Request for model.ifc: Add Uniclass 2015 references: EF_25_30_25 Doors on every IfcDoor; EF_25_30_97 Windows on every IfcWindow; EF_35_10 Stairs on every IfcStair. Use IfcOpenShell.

First a look at what the model holds.

```python
import ifcopenshell

model = ifcopenshell.open("model.ifc")
print(model.schema)
print("classifications:", [c.Name for c in model.by_type("IfcClassification")])
for ifc_class in ("IfcDoor", "IfcRoof", "IfcStair", "IfcWall", "IfcWindow"):
    print(ifc_class, len(model.by_type(ifc_class)))
```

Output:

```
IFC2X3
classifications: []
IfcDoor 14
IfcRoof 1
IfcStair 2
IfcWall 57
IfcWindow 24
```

```python
import ifcopenshell
import ifcopenshell.api.classification

model = ifcopenshell.open("model.ifc")

# IFC2X3 requires Source and Edition and has no link from the project to the system.
system = model.create_entity("IfcClassification", Source="NBS", Edition="2015", Name="Uniclass 2015")

codes = {
    "IfcDoor": ("EF_25_30_25", "Doors"),
    "IfcWindow": ("EF_25_30_97", "Windows"),
    "IfcStair": ("EF_35_10", "Stairs"),
}
for ifc_class, (code, name) in codes.items():
    products = model.by_type(ifc_class)
    ifcopenshell.api.classification.add_reference(
        model, products=products, classification=system, identification=code, name=name
    )
    print(code, len(products))

model.write("model_edited.ifc")
```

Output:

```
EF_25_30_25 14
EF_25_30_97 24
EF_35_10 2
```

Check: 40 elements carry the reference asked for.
